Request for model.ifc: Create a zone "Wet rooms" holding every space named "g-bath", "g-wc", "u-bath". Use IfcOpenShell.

First a look at what the model holds.

```python
import ifcopenshell

model = ifcopenshell.open("model.ifc")
print(model.schema)
seen = {}
for space in model.by_type("IfcSpace"):
    seen[space.LongName] = seen.get(space.LongName, 0) + 1
for name, count in sorted(seen.items(), key=str):
    print(count, "x", name)
print("zones:", [z.Name for z in model.by_type("IfcZone")][:20])
```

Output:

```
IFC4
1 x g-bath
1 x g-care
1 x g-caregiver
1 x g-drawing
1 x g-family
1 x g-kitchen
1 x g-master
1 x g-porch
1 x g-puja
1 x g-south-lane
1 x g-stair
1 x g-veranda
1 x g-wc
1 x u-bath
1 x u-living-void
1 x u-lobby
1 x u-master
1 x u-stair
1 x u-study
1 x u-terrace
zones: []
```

```python
import ifcopenshell
import ifcopenshell.api.group
import ifcopenshell.api.root

model = ifcopenshell.open("model.ifc")

names = {"g-bath", "g-wc", "u-bath"}
spaces = [s for s in model.by_type("IfcSpace") if s.LongName in names]

zone = ifcopenshell.api.root.create_entity(model, ifc_class="IfcZone", name="Wet rooms")
ifcopenshell.api.group.assign_group(model, products=spaces, group=zone)
print(len(spaces), "spaces in", zone.Name)

model.write("model_updated.ifc")
```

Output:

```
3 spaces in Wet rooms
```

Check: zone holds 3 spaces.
